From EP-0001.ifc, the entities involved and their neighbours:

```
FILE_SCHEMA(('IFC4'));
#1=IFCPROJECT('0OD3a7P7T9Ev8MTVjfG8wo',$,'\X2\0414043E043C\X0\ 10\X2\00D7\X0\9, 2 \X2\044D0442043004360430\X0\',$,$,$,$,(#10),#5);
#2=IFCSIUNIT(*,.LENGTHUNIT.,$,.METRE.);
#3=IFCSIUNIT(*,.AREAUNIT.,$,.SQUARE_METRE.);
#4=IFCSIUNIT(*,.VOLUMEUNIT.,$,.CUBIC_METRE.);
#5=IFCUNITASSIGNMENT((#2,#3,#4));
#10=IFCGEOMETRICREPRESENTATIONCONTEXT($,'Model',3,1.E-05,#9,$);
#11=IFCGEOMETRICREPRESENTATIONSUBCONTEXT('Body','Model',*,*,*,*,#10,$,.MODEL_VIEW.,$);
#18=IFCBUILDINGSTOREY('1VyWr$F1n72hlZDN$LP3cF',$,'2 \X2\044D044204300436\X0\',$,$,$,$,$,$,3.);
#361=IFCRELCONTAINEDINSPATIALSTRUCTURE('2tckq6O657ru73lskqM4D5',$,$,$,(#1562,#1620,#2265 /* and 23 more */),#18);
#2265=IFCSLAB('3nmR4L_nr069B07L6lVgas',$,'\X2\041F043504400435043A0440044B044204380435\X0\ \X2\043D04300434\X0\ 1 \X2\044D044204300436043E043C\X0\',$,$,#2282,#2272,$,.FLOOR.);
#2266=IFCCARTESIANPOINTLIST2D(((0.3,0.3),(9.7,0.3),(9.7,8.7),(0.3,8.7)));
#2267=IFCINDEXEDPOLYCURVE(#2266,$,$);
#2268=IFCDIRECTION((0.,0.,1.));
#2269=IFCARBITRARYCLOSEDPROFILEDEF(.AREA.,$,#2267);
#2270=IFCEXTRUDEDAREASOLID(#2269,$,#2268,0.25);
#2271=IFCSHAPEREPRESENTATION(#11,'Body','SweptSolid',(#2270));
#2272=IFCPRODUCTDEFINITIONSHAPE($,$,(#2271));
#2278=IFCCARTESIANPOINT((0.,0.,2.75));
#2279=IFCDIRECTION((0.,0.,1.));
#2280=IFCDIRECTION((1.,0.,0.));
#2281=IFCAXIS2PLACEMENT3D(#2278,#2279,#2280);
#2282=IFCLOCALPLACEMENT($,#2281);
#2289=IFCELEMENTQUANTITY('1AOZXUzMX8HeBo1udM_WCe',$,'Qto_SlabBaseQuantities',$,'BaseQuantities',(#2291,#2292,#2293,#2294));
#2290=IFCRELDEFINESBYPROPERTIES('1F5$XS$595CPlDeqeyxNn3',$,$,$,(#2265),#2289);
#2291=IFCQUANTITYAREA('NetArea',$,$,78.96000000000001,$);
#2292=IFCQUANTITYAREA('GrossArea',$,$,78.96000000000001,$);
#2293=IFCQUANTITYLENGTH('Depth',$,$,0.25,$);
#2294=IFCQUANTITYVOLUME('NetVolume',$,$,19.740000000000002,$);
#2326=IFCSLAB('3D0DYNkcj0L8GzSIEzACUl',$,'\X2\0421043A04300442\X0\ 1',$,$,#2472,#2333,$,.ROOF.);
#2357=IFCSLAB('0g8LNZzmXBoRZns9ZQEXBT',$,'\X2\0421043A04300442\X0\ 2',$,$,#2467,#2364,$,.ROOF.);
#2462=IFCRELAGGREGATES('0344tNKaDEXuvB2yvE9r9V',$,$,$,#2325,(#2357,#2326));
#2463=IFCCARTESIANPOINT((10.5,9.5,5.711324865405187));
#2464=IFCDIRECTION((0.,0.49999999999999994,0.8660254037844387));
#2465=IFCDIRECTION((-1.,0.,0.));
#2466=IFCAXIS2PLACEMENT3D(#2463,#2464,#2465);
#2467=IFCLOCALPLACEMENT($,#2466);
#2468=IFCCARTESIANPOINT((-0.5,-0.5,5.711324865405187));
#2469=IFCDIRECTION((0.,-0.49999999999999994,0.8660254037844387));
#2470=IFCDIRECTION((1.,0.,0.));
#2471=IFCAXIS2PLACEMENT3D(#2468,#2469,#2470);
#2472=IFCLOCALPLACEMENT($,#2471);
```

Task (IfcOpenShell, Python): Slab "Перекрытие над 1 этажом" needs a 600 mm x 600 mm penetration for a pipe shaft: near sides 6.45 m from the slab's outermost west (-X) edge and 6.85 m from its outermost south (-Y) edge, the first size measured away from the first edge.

```python
import numpy as np
import ifcopenshell
import ifcopenshell.api.feature
import ifcopenshell.api.geometry
import ifcopenshell.api.pset
import ifcopenshell.api.root
import ifcopenshell.geom
import ifcopenshell.util.element
import ifcopenshell.util.placement
import ifcopenshell.util.representation
import ifcopenshell.util.shape
import ifcopenshell.util.unit

model = ifcopenshell.open("EP-0001.ifc")
unit_scale = ifcopenshell.util.unit.calculate_unit_scale(model)
area_scale = ifcopenshell.util.unit.calculate_unit_scale(model, "AREAUNIT")
volume_scale = ifcopenshell.util.unit.calculate_unit_scale(model, "VOLUMEUNIT")
settings = ifcopenshell.geom.settings()


def volume(element):
    """Net volume in cubic metres, openings subtracted."""
    shape = ifcopenshell.geom.create_shape(settings, element)
    return ifcopenshell.util.shape.get_volume(shape.geometry)


slab = model.by_guid("3nmR4L_nr069B07L6lVgas")
before = volume(slab)

# Extent in the slab's own axes, in metres. The edges named are its -X and -Y sides.
slab_shape = ifcopenshell.geom.create_shape(settings, slab)
vertices = ifcopenshell.util.shape.get_vertices(slab_shape.geometry)
x_min, y_min, bottom = vertices.min(axis=0)
top = vertices[:, 2].max()

opening = ifcopenshell.api.root.create_entity(model, ifc_class="IfcOpeningElement", name="Pipe shaft opening", predefined_type="OPENING")
context = ifcopenshell.util.representation.get_context(model, "Model", "Body", "MODEL_VIEW")
width, depth = 0.6, 0.6
outline = [(0.0, 0.0), (width, 0.0), (width, depth), (0.0, depth), (0.0, 0.0)]
# Overshoot both faces by 50 mm so the cut is clean.
shape = ifcopenshell.api.geometry.add_slab_representation(
    model, context=context, depth=top - bottom + 0.1, polyline=outline
)
ifcopenshell.api.geometry.assign_representation(model, product=opening, representation=shape)

matrix = ifcopenshell.util.placement.get_local_placement(slab.ObjectPlacement)
matrix[:, 3] = matrix @ np.append(np.array([x_min + 6.45, y_min + 6.85, bottom - 0.05]) / unit_scale, 1.0)
ifcopenshell.api.geometry.edit_object_placement(model, product=opening, matrix=matrix, is_si=False)
ifcopenshell.api.feature.add_feature(model, feature=opening, element=slab)

after = volume(slab)

# Update the slab's stored quantities.
qto = model.by_id(ifcopenshell.util.element.get_pset(slab, "Qto_SlabBaseQuantities", should_inherit=False)["id"])
ifcopenshell.api.pset.edit_qto(model, qto=qto, properties={
    "NetArea": after / (top - bottom) / area_scale,
    "NetVolume": after / volume_scale,
})

print(f"slab volume {before:.3f} -> {after:.3f} m3")

model.write("EP-0001-out.ifc")
```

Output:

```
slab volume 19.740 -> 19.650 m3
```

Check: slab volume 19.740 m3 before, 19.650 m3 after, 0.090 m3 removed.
